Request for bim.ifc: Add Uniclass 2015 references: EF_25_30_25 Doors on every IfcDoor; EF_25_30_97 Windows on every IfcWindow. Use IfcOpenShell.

First a look at what the model holds.

```python
import ifcopenshell

model = ifcopenshell.open("bim.ifc")
print(model.schema)
print("classifications:", [c.Name for c in model.by_type("IfcClassification")])
for ifc_class in ("IfcDoor", "IfcRoof", "IfcStair", "IfcWall", "IfcWindow"):
    print(ifc_class, len(model.by_type(ifc_class)))
```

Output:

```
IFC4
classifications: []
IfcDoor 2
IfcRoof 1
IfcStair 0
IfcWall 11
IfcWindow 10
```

```python
import ifcopenshell
import ifcopenshell.api.classification

model = ifcopenshell.open("bim.ifc")

system = ifcopenshell.api.classification.add_classification(model, classification="Uniclass 2015")

codes = {
    "IfcDoor": ("EF_25_30_25", "Doors"),
    "IfcWindow": ("EF_25_30_97", "Windows"),
}
for ifc_class, (code, name) in codes.items():
    products = model.by_type(ifc_class)
    ifcopenshell.api.classification.add_reference(
        model, products=products, classification=system, identification=code, name=name
    )
    print(code, len(products))

model.write("bim-out.ifc")
```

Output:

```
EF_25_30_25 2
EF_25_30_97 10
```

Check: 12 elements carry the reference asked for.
